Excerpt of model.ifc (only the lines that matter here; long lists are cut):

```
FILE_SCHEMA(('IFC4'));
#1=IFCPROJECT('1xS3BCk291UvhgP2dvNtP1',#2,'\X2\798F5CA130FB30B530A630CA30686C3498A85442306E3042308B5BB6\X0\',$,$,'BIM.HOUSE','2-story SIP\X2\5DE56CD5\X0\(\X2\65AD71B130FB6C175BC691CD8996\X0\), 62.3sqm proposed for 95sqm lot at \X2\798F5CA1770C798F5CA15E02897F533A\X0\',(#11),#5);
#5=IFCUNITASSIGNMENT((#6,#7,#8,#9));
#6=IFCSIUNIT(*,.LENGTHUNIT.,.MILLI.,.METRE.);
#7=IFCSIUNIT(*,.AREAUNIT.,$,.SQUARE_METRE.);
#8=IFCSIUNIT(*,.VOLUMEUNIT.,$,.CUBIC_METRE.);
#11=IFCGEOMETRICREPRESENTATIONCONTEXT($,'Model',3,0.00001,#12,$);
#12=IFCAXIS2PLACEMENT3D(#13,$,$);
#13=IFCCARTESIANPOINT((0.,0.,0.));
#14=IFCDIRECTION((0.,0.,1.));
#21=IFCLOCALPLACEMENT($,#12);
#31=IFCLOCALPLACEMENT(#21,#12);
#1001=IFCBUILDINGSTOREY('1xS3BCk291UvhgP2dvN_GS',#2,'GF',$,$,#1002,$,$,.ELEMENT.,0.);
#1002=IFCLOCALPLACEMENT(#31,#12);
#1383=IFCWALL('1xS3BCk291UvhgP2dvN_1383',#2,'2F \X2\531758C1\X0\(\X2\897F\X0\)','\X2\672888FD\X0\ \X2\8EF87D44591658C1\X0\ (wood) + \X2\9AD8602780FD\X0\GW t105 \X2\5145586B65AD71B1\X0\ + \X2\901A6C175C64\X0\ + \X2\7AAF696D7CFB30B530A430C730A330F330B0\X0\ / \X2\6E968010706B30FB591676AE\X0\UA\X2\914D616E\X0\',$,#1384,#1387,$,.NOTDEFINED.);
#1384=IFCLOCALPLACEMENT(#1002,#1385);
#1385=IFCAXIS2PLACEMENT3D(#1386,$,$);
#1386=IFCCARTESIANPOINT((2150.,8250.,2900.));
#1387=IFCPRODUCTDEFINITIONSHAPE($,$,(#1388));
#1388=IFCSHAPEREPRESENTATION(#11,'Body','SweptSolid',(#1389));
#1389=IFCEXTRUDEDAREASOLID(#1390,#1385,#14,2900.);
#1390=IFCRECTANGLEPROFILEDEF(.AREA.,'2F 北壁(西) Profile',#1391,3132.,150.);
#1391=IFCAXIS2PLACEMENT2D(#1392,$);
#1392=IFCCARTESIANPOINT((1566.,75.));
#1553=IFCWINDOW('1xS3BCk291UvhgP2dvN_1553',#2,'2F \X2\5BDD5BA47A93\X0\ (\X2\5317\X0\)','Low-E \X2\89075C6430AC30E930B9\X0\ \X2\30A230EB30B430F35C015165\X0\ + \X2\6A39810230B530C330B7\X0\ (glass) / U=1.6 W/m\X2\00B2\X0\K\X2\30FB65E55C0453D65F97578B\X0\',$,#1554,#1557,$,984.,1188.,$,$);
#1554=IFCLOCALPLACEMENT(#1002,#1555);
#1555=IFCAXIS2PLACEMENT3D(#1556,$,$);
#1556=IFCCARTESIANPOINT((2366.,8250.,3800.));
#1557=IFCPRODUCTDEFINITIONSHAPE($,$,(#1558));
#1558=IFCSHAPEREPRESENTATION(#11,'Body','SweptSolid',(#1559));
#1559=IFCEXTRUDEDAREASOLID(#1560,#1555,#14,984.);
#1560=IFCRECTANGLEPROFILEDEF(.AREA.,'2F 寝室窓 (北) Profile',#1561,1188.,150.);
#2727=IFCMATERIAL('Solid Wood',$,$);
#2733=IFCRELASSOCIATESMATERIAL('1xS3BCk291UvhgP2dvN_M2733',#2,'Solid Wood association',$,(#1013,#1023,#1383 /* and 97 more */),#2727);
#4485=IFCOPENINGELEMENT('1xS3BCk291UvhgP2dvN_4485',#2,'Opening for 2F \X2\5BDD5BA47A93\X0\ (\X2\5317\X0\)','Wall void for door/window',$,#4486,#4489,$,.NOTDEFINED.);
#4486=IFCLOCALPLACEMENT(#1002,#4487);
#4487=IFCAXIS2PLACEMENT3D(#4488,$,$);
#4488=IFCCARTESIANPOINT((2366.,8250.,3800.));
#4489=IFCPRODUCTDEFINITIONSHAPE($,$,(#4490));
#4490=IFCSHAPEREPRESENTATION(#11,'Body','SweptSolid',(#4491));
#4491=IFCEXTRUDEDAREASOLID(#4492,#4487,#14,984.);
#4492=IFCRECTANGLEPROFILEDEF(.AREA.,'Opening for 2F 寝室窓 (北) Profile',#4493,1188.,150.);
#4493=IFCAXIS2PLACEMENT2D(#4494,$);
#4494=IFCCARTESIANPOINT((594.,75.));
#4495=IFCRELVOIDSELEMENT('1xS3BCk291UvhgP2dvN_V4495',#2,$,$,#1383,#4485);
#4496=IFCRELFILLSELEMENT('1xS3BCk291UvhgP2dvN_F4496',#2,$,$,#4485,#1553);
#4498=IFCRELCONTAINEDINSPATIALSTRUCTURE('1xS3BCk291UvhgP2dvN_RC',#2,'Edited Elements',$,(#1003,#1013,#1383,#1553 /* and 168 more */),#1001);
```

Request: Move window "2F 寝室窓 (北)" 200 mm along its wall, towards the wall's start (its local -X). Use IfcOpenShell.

```python
import ifcopenshell
import ifcopenshell.api.geometry
import ifcopenshell.util.placement
import ifcopenshell.util.unit

model = ifcopenshell.open("model.ifc")
unit_scale = ifcopenshell.util.unit.calculate_unit_scale(model)

window = model.by_guid("1xS3BCk291UvhgP2dvN_1553")
opening = window.FillsVoids[0].RelatingOpeningElement
wall = opening.VoidsElements[0].RelatingBuildingElement

wall_matrix = ifcopenshell.util.placement.get_local_placement(wall.ObjectPlacement)
shift = wall_matrix[:3, 0] * -0.2 / unit_scale
before = ifcopenshell.util.placement.get_local_placement(window.ObjectPlacement)[:3, 3].copy()

# The window is not placed relative to its opening, so move both.
for product in (opening, window):
    matrix = ifcopenshell.util.placement.get_local_placement(product.ObjectPlacement)
    matrix[:3, 3] += shift
    ifcopenshell.api.geometry.edit_object_placement(model, product=product, matrix=matrix, is_si=False)

after = ifcopenshell.util.placement.get_local_placement(window.ObjectPlacement)[:3, 3]
print("window moved by", (after - before).round(3) + 0.0)

model.write("model_updated.ifc")
```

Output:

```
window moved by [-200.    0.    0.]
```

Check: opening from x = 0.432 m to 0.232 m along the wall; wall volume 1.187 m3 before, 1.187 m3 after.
